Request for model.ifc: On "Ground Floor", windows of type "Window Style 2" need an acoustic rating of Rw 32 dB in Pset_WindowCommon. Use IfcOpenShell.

First a look at what the model holds.

```python
import ifcopenshell
import ifcopenshell.util.element

model = ifcopenshell.open("model.ifc")
print(model.schema)
storey = next(s for s in model.by_type("IfcBuildingStorey") if s.Name == "Ground Floor")
windows = [e for e in ifcopenshell.util.element.get_decomposition(storey) if e.is_a("IfcWindow")]
seen = {}
for e in windows:
    element_type = ifcopenshell.util.element.get_type(e)
    key = (element_type.Name if element_type != e and element_type else None, ifcopenshell.util.element.get_pset(e, "Pset_WindowCommon", "AcousticRating"))
    seen[key] = seen.get(key, 0) + 1
for (name, value), count in sorted(seen.items(), key=str):
    print(count, "x", name, "|", value)
```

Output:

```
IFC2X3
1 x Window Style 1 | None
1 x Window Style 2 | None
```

```python
import ifcopenshell
import ifcopenshell.api.pset
import ifcopenshell.util.element

model = ifcopenshell.open("model.ifc")

storey = next(s for s in model.by_type("IfcBuildingStorey") if s.Name == "Ground Floor")
windows = [e for e in ifcopenshell.util.element.get_decomposition(storey) if e.is_a("IfcWindow")]

count = 0
for e in windows:
    element_type = ifcopenshell.util.element.get_type(e)
    if element_type in (None, e) or element_type.Name != "Window Style 2":
        continue
    # add_pset returns the element's existing set when there is one.
    pset = ifcopenshell.api.pset.add_pset(model, product=e, name="Pset_WindowCommon")
    ifcopenshell.api.pset.edit_pset(model, pset=pset, properties={"AcousticRating": "Rw 32 dB"})
    count += 1

print(count, "windows updated")

model.write("model_edited.ifc")
```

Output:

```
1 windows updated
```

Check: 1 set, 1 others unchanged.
